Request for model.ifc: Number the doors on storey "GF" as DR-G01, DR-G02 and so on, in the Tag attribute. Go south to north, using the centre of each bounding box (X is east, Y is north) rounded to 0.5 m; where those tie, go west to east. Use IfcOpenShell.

First a look at what the model holds.

```python
import ifcopenshell
import ifcopenshell.util.element
import ifcopenshell.util.placement

model = ifcopenshell.open("model.ifc")
print(model.schema)
storey = next(s for s in model.by_type("IfcBuildingStorey") if s.Name == "GF")
doors = [e for e in ifcopenshell.util.element.get_decomposition(storey) if e.is_a("IfcDoor")]
for e in sorted(doors, key=lambda e: e.id()):
    origin = ifcopenshell.util.placement.get_local_placement(e.ObjectPlacement)[:3, 3]
    print(e.id(), e.Tag, e.Name, origin.round(2) + 0.0, sep=" | ")
```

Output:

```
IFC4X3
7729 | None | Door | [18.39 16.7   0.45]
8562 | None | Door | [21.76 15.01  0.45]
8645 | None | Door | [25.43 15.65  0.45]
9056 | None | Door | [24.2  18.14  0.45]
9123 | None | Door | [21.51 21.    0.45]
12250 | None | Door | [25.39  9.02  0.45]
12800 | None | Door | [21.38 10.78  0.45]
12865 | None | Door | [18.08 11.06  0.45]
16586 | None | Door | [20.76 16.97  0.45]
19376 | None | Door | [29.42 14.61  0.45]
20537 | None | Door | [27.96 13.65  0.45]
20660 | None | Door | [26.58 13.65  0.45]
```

```python
import ifcopenshell
import ifcopenshell.geom
import ifcopenshell.util.element
import ifcopenshell.util.shape

model = ifcopenshell.open("model.ifc")
settings = ifcopenshell.geom.settings()
settings.set("use-world-coords", True)


def centre(element):
    shape = ifcopenshell.geom.create_shape(settings, element)
    return ifcopenshell.util.shape.get_bbox_centroid(shape.geometry)


storey = next(s for s in model.by_type("IfcBuildingStorey") if s.Name == "GF")
doors = [e for e in ifcopenshell.util.element.get_decomposition(storey) if e.is_a("IfcDoor")]

# Insertion points can sit at a corner or the storey origin, so sort by the geometry (in metres).
centres = {e: centre(e) for e in doors}
doors.sort(key=lambda e: (round(centres[e][1] / 0.5), centres[e][0]))

for i, e in enumerate(doors, start=1):
    number = f"DR-G{i:02d}"
    e.Tag = number
    print(e.id(), number)

model.write("model_rev.ifc")
```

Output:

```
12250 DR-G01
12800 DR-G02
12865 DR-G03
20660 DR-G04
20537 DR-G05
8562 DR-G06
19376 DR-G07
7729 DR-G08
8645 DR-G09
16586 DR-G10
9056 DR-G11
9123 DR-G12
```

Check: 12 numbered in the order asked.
